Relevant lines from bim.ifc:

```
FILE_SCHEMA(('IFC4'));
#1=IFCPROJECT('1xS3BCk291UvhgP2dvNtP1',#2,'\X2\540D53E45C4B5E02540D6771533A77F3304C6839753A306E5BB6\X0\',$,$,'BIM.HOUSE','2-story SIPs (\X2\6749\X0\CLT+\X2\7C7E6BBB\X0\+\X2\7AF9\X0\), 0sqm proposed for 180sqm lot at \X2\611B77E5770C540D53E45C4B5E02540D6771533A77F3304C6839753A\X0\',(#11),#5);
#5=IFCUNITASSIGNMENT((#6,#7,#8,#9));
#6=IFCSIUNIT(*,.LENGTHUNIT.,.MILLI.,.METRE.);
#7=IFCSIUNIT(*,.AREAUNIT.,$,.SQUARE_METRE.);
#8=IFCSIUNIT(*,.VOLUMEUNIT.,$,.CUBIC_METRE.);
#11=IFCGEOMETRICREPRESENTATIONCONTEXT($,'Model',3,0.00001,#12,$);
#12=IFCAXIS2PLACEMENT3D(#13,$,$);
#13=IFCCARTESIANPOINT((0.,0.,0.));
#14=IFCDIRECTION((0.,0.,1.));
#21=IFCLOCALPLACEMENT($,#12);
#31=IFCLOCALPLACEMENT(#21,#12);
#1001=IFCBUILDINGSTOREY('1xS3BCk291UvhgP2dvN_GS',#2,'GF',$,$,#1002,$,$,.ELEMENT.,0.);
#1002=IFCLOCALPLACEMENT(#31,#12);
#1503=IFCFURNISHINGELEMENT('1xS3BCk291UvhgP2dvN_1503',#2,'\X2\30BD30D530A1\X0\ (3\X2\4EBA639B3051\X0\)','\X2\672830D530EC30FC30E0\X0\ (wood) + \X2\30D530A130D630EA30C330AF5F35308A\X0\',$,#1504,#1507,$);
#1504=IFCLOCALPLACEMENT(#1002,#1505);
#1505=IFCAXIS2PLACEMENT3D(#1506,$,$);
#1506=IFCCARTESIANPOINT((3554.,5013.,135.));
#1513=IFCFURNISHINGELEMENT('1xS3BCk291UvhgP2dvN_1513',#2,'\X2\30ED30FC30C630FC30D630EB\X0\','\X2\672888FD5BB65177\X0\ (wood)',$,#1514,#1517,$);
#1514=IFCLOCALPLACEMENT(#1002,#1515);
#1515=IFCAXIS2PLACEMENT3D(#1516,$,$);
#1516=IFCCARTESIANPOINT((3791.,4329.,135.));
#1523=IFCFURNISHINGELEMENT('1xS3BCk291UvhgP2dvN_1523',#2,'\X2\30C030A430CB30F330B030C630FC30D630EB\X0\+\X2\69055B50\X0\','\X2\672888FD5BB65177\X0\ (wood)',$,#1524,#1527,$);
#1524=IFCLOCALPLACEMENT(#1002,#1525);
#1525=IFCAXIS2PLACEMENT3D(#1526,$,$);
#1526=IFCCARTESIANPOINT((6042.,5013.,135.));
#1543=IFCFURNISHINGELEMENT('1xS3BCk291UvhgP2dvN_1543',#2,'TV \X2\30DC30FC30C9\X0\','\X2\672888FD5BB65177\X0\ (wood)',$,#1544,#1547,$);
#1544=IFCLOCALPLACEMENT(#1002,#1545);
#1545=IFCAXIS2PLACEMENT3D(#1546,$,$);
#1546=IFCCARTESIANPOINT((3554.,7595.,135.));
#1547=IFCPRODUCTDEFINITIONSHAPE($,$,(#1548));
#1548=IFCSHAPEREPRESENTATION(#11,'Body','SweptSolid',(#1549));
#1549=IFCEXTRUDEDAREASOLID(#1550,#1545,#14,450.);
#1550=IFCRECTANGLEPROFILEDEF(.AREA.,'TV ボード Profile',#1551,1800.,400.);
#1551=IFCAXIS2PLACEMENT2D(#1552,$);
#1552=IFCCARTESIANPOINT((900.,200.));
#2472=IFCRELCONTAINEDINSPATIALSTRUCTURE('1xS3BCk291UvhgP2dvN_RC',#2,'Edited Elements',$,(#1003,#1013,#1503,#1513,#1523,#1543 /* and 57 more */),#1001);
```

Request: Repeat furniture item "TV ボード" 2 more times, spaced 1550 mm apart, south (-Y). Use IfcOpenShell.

```python
import numpy as np
import ifcopenshell
import ifcopenshell.api.geometry
import ifcopenshell.api.root
import ifcopenshell.util.element
import ifcopenshell.util.placement
import ifcopenshell.util.unit

model = ifcopenshell.open("bim.ifc")
unit_scale = ifcopenshell.util.unit.calculate_unit_scale(model)


def reuse_history(source, copy):
    """copy_class also copies each property set's owner history, people and application; keep the originals."""
    for rel in copy.IsDefinedBy:
        if rel.is_a("IfcRelDefinesByProperties") and (history := rel.RelatingPropertyDefinition.OwnerHistory):
            rel.RelatingPropertyDefinition.OwnerHistory = source.OwnerHistory
            ifcopenshell.util.element.remove_deep2(model, history)


source = model.by_guid("1xS3BCk291UvhgP2dvN_1543")
base = ifcopenshell.util.placement.get_local_placement(source.ObjectPlacement)
step = np.array([0.0, -1.0, 0.0]) * 1.55 / unit_scale

for i in range(1, 3):
    copy = ifcopenshell.api.root.copy_class(model, product=source)
    copy.Representation = ifcopenshell.util.element.copy_deep(
        model, source.Representation, exclude=["IfcGeometricRepresentationContext", "IfcRepresentationMap"]
    )
    reuse_history(source, copy)
    matrix = base.copy()
    matrix[:3, 3] += i * step
    print("added at", matrix[:3, 3].round(3) + 0.0)
    ifcopenshell.api.geometry.edit_object_placement(model, product=copy, matrix=matrix, is_si=False)

model.write("bim_rev.ifc")
```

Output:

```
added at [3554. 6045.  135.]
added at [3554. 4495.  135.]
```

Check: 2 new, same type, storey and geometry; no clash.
